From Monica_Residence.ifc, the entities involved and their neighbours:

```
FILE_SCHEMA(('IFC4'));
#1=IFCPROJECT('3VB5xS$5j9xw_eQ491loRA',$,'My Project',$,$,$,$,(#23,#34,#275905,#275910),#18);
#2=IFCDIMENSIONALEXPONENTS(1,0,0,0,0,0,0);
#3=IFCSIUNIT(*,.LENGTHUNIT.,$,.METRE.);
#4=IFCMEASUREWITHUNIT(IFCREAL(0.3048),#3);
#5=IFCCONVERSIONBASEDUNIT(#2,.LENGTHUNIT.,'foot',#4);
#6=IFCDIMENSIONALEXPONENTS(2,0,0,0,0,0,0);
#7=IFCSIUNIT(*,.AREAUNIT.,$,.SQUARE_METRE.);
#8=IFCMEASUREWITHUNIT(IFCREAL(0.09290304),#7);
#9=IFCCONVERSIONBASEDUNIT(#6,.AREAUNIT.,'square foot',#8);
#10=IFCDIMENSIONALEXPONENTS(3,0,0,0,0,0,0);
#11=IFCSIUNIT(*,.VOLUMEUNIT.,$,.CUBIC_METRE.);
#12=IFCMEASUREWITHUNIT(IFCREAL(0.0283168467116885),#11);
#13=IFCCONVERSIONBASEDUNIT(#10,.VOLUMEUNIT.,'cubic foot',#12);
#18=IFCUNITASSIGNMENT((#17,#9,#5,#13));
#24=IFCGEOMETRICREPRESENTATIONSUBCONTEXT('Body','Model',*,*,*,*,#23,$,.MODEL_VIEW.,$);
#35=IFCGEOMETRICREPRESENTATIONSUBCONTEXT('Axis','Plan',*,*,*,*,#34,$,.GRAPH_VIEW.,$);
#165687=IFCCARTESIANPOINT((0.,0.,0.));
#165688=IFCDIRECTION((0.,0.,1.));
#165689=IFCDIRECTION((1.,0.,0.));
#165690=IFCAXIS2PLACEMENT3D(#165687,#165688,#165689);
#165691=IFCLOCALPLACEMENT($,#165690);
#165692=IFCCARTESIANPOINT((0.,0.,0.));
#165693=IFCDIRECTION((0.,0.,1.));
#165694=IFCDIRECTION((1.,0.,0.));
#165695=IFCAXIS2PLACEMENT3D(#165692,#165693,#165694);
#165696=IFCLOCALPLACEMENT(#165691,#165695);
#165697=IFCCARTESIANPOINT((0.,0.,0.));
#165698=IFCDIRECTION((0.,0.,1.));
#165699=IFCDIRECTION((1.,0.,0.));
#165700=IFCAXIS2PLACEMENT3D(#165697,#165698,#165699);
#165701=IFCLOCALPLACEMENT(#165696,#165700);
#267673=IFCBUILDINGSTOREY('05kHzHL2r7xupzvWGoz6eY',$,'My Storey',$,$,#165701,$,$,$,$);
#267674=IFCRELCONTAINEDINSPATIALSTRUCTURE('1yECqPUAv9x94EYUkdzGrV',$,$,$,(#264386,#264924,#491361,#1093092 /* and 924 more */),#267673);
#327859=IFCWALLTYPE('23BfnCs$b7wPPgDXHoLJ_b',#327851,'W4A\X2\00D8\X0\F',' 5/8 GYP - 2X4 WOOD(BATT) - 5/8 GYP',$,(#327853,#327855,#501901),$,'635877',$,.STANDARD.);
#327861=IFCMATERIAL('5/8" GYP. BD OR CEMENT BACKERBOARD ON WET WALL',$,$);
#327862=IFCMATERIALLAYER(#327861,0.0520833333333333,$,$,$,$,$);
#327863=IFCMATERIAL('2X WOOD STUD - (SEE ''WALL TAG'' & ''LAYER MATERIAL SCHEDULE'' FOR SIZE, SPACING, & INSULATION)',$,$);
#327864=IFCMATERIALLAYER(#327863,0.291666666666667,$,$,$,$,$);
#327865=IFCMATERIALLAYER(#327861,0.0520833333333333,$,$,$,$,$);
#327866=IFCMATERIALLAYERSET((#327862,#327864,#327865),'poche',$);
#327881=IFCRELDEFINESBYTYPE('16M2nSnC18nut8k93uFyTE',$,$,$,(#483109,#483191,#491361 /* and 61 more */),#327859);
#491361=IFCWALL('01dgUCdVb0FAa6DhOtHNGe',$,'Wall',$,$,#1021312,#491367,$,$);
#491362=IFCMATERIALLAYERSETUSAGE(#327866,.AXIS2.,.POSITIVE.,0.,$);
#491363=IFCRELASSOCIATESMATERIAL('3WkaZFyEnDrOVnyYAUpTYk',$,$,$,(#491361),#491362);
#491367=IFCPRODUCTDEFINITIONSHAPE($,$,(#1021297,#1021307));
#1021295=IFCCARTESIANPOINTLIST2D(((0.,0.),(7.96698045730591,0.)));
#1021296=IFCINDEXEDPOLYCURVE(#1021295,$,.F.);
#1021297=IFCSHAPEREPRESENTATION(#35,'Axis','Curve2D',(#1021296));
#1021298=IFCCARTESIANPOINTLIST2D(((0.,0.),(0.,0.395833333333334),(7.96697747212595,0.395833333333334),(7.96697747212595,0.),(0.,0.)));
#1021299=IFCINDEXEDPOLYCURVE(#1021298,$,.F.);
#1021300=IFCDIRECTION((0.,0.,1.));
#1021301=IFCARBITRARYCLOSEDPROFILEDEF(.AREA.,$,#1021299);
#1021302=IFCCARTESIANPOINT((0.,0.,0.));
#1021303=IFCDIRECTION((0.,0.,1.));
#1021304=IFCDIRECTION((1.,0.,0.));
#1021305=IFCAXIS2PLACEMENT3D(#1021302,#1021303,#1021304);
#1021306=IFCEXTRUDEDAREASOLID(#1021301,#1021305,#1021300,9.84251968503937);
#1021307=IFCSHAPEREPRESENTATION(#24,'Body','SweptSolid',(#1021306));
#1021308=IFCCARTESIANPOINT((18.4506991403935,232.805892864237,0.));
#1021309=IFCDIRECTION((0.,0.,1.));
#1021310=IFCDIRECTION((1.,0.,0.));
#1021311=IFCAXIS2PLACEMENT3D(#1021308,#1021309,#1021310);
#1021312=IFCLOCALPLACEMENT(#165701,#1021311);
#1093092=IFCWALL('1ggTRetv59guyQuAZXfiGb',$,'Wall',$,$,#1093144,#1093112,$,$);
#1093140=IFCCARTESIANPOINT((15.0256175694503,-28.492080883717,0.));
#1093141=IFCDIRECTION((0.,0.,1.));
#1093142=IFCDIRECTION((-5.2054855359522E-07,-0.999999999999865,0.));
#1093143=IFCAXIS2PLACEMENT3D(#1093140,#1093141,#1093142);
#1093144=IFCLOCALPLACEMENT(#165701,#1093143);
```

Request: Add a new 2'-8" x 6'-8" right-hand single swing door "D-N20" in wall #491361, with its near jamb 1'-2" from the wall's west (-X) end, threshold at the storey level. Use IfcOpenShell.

```python
import numpy as np
import ifcopenshell
import ifcopenshell.api.feature
import ifcopenshell.api.geometry
import ifcopenshell.api.root
import ifcopenshell.api.spatial
import ifcopenshell.geom
import ifcopenshell.util.element
import ifcopenshell.util.placement
import ifcopenshell.util.representation
import ifcopenshell.util.shape
import ifcopenshell.util.unit

model = ifcopenshell.open("Monica_Residence.ifc")
unit_scale = ifcopenshell.util.unit.calculate_unit_scale(model)
settings = ifcopenshell.geom.settings()


def volume(element):
    """Net volume in cubic metres, openings subtracted."""
    shape = ifcopenshell.geom.create_shape(settings, element)
    return ifcopenshell.util.shape.get_volume(shape.geometry)


wall = model.by_guid("01dgUCdVb0FAa6DhOtHNGe")
storey = ifcopenshell.util.element.get_container(wall, ifc_class="IfcBuildingStorey")
context = ifcopenshell.util.representation.get_context(model, "Model", "Body", "MODEL_VIEW")
before = volume(wall)

width, height, from_end, sill = 0.8128, 2.032, 0.3556, 0.0  # metres

# The wall runs along its own X axis, and the end named is its -X end.
wall_shape = ifcopenshell.geom.create_shape(settings, wall)
x, y, z = ifcopenshell.util.shape.get_vertices(wall_shape.geometry).T
start = x.min() + from_end
face, thickness = float(y.min()), float(y.max() - y.min())
wall_matrix = ifcopenshell.util.placement.get_local_placement(wall.ObjectPlacement)
level = ifcopenshell.util.placement.get_local_placement(storey.ObjectPlacement)[2, 3]


def in_wall(x, y):
    """Placement at x, y metres in the wall's axes, at sill height."""
    matrix = wall_matrix.copy()
    matrix[:, 3] = wall_matrix @ np.array([x / unit_scale, y / unit_scale, 0.0, 1.0])
    matrix[2, 3] = level + sill / unit_scale
    return matrix


# Opening: a box that overshoots both wall faces by 50 mm.
opening = ifcopenshell.api.root.create_entity(model, ifc_class="IfcOpeningElement", predefined_type="OPENING")
box = ifcopenshell.api.geometry.add_wall_representation(
    model, context=context, length=width, height=height, thickness=thickness + 0.1
)
ifcopenshell.api.geometry.assign_representation(model, product=opening, representation=box)
ifcopenshell.api.geometry.edit_object_placement(model, product=opening, matrix=in_wall(start, face - 0.05), is_si=False)
ifcopenshell.api.feature.add_feature(model, feature=opening, element=wall)

door = ifcopenshell.api.root.create_entity(model, ifc_class="IfcDoor", name="D-N20", predefined_type="DOOR")
door.OverallWidth, door.OverallHeight = width / unit_scale, height / unit_scale
door.OperationType = "SINGLE_SWING_RIGHT"
body = ifcopenshell.api.geometry.add_door_representation(
    model,
    context=context,
    overall_width=door.OverallWidth,
    overall_height=door.OverallHeight,
    operation_type="SINGLE_SWING_RIGHT",
    lining_properties={"LiningDepth": thickness / unit_scale, "ThresholdDepth": thickness / unit_scale},
)
ifcopenshell.api.geometry.assign_representation(model, product=door, representation=body)
ifcopenshell.api.spatial.assign_container(model, products=[door], relating_structure=storey)
ifcopenshell.api.feature.add_filling(model, opening=opening, element=door)

# The lining spans the wall, so the door starts at the wall face.
ifcopenshell.api.geometry.edit_object_placement(model, product=door, matrix=in_wall(start, face), is_si=False)

after = volume(wall)

print(f"wall volume {before:.3f} -> {after:.3f} m3")

model.write("Monica_Residence_edited.ifc")
```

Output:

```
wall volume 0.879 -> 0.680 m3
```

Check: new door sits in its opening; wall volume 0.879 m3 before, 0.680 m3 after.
